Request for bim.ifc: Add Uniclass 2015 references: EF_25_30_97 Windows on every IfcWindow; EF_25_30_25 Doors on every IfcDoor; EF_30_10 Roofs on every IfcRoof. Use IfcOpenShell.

First a look at what the model holds.

```python
import ifcopenshell

model = ifcopenshell.open("bim.ifc")
print(model.schema)
print("classifications:", [c.Name for c in model.by_type("IfcClassification")])
for ifc_class in ("IfcDoor", "IfcRoof", "IfcStair", "IfcWall", "IfcWindow"):
    print(ifc_class, len(model.by_type(ifc_class)))
```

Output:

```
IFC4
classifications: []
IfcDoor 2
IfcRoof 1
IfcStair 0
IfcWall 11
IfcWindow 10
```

```python
import ifcopenshell
import ifcopenshell.api.classification

model = ifcopenshell.open("bim.ifc")

system = ifcopenshell.api.classification.add_classification(model, classification="Uniclass 2015")

codes = {
    "IfcWindow": ("EF_25_30_97", "Windows"),
    "IfcDoor": ("EF_25_30_25", "Doors"),
    "IfcRoof": ("EF_30_10", "Roofs"),
}
for ifc_class, (code, name) in codes.items():
    products = model.by_type(ifc_class)
    ifcopenshell.api.classification.add_reference(
        model, products=products, classification=system, identification=code, name=name
    )
    print(code, len(products))

model.write("bim_updated.ifc")
```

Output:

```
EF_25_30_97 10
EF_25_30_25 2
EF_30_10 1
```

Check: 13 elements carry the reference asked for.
